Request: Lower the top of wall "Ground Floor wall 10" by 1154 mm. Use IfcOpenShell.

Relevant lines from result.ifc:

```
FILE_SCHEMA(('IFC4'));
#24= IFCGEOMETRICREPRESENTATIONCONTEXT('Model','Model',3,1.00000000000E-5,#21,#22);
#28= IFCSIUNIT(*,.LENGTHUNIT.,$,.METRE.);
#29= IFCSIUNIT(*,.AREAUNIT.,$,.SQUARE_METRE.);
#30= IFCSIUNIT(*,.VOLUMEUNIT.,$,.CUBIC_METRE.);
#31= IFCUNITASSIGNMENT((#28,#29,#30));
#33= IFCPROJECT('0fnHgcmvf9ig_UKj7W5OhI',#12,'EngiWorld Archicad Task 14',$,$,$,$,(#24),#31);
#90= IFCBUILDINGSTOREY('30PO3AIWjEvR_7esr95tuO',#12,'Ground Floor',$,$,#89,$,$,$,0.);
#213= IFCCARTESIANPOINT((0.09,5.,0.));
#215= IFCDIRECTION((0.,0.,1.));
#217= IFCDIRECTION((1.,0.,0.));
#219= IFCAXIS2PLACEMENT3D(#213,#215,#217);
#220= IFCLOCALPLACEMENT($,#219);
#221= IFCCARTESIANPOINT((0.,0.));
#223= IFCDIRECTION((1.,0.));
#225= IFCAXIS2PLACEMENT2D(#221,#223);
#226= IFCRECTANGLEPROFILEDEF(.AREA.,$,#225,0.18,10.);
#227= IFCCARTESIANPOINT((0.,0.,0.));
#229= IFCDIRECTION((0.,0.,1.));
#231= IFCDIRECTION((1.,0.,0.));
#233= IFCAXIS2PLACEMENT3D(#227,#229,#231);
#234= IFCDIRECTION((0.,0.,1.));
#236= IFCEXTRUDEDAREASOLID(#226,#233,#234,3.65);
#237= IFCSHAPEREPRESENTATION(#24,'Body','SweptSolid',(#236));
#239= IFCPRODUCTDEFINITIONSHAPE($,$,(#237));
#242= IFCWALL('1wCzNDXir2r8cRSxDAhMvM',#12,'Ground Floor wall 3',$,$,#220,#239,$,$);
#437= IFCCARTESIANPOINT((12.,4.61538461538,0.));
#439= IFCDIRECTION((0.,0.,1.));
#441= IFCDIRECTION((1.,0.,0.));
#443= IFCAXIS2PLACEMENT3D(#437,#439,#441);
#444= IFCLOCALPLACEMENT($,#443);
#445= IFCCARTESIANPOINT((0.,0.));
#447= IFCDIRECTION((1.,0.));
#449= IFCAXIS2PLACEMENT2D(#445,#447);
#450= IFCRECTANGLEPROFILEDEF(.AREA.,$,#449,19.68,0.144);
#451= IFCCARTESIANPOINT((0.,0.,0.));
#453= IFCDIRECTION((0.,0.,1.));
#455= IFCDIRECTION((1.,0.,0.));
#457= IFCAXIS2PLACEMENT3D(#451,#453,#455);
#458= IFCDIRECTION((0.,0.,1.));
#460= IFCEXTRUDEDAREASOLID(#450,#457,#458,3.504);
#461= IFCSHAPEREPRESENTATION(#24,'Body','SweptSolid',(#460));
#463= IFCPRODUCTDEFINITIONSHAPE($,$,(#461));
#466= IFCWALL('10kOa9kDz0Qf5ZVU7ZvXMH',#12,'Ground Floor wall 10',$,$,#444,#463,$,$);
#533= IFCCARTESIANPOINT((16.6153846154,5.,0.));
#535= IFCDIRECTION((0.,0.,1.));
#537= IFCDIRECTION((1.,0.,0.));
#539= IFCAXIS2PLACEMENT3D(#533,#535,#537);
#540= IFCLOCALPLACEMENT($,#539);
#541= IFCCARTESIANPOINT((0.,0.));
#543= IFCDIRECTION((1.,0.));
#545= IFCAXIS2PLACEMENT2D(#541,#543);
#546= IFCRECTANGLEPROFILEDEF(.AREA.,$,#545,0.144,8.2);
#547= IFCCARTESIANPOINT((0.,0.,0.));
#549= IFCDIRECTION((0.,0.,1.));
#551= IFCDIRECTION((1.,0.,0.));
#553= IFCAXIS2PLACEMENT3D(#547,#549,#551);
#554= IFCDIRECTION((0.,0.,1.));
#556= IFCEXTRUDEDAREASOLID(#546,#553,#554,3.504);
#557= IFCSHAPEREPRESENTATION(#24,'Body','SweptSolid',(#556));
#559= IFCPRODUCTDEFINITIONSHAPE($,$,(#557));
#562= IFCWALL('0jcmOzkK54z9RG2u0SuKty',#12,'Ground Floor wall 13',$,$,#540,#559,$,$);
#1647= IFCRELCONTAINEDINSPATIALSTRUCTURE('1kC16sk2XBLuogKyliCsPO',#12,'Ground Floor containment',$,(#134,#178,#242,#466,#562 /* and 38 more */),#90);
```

```python
import ifcopenshell
import ifcopenshell.geom
import ifcopenshell.util.shape

model = ifcopenshell.open("result.ifc")
settings = ifcopenshell.geom.settings()


def volume(element):
    """Net volume in cubic metres, openings subtracted."""
    shape = ifcopenshell.geom.create_shape(settings, element)
    return ifcopenshell.util.shape.get_volume(shape.geometry)


wall = model.by_guid("10kOa9kDz0Qf5ZVU7ZvXMH")
before = volume(wall)

body = next(r for r in wall.Representation.Representations if r.RepresentationIdentifier == "Body")
solid = body.Items[0]
old_height = solid.Depth
solid.Depth -= 1.154
after = volume(wall)

print(f"height {old_height:g} -> {solid.Depth:g}, volume {before:.3f} -> {after:.3f} m3")

model.write("result_rev.ifc")
```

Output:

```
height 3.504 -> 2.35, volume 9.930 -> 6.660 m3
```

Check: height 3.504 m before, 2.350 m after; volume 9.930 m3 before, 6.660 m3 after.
